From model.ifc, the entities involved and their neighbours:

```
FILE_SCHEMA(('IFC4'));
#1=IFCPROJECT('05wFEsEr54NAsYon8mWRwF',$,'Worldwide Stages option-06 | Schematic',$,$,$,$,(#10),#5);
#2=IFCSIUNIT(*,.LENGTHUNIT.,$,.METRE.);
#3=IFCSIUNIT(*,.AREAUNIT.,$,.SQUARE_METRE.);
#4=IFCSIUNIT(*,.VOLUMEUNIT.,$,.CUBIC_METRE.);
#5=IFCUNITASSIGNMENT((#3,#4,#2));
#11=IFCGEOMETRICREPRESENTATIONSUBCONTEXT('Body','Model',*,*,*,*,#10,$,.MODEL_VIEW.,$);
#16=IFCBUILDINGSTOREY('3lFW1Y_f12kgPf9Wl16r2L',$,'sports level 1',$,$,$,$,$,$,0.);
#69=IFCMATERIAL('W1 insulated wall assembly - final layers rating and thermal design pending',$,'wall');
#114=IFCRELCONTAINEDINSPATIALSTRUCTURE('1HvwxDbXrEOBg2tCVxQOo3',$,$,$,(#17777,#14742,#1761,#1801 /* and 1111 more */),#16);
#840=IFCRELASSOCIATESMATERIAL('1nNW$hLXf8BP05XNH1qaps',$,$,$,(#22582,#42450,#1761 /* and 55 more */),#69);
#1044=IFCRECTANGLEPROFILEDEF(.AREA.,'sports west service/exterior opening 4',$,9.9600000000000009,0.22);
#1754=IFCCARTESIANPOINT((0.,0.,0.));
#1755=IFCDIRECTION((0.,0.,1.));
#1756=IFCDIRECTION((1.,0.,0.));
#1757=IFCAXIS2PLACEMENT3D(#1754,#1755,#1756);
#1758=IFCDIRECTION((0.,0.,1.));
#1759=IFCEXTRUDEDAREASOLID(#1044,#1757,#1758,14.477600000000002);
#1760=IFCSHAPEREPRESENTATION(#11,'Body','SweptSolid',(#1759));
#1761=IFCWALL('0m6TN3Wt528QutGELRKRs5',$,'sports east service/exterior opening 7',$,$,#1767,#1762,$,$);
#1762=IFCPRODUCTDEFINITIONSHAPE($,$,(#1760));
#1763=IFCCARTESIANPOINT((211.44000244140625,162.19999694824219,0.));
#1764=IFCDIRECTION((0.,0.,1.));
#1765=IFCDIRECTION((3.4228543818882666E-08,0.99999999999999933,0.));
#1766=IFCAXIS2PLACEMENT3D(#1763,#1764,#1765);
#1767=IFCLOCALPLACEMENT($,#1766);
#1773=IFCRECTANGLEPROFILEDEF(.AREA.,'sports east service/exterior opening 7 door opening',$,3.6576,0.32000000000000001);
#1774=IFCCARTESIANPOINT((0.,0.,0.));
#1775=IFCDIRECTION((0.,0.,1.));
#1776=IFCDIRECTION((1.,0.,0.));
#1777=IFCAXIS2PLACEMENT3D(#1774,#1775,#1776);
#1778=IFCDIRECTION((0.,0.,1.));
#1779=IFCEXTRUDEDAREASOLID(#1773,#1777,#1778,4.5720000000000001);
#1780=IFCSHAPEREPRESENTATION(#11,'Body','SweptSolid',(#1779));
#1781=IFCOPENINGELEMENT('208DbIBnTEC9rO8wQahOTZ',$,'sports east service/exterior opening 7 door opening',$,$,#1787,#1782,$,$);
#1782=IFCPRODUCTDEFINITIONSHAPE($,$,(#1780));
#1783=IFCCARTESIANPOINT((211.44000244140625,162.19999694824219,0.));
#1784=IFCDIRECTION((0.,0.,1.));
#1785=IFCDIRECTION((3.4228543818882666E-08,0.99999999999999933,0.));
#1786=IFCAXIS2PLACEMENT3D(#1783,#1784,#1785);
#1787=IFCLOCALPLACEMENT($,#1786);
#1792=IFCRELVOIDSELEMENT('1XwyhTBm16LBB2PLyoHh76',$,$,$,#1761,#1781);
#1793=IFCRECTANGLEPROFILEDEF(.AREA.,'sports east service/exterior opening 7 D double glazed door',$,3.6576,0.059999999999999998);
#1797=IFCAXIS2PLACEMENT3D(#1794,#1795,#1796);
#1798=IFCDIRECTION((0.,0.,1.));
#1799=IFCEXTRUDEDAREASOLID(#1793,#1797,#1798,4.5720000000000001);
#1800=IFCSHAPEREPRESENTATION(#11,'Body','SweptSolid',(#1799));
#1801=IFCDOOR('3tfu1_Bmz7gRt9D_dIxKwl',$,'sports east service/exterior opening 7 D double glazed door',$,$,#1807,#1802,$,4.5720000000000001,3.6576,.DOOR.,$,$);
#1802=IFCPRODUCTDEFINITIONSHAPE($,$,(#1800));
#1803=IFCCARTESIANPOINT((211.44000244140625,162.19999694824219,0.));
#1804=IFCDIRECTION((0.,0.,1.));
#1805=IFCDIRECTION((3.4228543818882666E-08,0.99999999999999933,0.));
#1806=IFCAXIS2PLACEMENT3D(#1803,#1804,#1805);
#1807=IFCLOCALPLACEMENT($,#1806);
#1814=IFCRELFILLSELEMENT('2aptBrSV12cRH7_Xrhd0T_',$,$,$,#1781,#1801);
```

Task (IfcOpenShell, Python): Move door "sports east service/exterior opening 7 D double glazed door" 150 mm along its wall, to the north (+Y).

```python
import ifcopenshell
import ifcopenshell.api.geometry
import ifcopenshell.util.placement
import ifcopenshell.util.unit

model = ifcopenshell.open("model.ifc")
unit_scale = ifcopenshell.util.unit.calculate_unit_scale(model)

door = model.by_id(1801)
opening = door.FillsVoids[0].RelatingOpeningElement
wall = opening.VoidsElements[0].RelatingBuildingElement

wall_matrix = ifcopenshell.util.placement.get_local_placement(wall.ObjectPlacement)
shift = wall_matrix[:3, 0] * 0.15 / unit_scale
before = ifcopenshell.util.placement.get_local_placement(door.ObjectPlacement)[:3, 3].copy()

# The door is not placed relative to its opening, so move both.
for product in (opening, door):
    matrix = ifcopenshell.util.placement.get_local_placement(product.ObjectPlacement)
    matrix[:3, 3] += shift
    ifcopenshell.api.geometry.edit_object_placement(model, product=product, matrix=matrix, is_si=False)

after = ifcopenshell.util.placement.get_local_placement(door.ObjectPlacement)[:3, 3]
print("door moved by", (after - before).round(3) + 0.0)

model.write("model_updated.ifc")
```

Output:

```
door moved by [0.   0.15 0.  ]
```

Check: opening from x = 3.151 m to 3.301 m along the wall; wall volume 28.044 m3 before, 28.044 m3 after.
